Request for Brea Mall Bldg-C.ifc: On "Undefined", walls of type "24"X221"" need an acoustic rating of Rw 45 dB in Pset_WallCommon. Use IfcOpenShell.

First a look at what the model holds.

```python
import ifcopenshell
import ifcopenshell.util.element

model = ifcopenshell.open("Brea Mall Bldg-C.ifc")
print(model.schema)
storey = next(s for s in model.by_type("IfcBuildingStorey") if s.Name == "Undefined")
walls = [e for e in ifcopenshell.util.element.get_decomposition(storey) if e.is_a("IfcWall")]
seen = {}
for e in walls:
    element_type = ifcopenshell.util.element.get_type(e)
    key = (element_type.Name if element_type != e and element_type else None, ifcopenshell.util.element.get_pset(e, "Pset_WallCommon", "AcousticRating"))
    seen[key] = seen.get(key, 0) + 1
for (name, value), count in sorted(seen.items(), key=str):
    print(count, "x", name, "|", value)
```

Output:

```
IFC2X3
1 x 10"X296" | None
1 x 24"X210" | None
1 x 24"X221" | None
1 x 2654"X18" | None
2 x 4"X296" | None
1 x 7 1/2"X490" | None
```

```python
import ifcopenshell
import ifcopenshell.api.pset
import ifcopenshell.util.element

model = ifcopenshell.open("Brea Mall Bldg-C.ifc")

storey = next(s for s in model.by_type("IfcBuildingStorey") if s.Name == "Undefined")
walls = [e for e in ifcopenshell.util.element.get_decomposition(storey) if e.is_a("IfcWall")]

count = 0
for e in walls:
    element_type = ifcopenshell.util.element.get_type(e)
    if element_type in (None, e) or element_type.Name != '24"X221"':
        continue
    # add_pset returns the element's existing set when there is one.
    pset = ifcopenshell.api.pset.add_pset(model, product=e, name="Pset_WallCommon")
    ifcopenshell.api.pset.edit_pset(model, pset=pset, properties={"AcousticRating": "Rw 45 dB"})
    count += 1

print(count, "walls updated")

model.write("Brea Mall Bldg-C_rev.ifc")
```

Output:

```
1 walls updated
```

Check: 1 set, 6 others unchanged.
